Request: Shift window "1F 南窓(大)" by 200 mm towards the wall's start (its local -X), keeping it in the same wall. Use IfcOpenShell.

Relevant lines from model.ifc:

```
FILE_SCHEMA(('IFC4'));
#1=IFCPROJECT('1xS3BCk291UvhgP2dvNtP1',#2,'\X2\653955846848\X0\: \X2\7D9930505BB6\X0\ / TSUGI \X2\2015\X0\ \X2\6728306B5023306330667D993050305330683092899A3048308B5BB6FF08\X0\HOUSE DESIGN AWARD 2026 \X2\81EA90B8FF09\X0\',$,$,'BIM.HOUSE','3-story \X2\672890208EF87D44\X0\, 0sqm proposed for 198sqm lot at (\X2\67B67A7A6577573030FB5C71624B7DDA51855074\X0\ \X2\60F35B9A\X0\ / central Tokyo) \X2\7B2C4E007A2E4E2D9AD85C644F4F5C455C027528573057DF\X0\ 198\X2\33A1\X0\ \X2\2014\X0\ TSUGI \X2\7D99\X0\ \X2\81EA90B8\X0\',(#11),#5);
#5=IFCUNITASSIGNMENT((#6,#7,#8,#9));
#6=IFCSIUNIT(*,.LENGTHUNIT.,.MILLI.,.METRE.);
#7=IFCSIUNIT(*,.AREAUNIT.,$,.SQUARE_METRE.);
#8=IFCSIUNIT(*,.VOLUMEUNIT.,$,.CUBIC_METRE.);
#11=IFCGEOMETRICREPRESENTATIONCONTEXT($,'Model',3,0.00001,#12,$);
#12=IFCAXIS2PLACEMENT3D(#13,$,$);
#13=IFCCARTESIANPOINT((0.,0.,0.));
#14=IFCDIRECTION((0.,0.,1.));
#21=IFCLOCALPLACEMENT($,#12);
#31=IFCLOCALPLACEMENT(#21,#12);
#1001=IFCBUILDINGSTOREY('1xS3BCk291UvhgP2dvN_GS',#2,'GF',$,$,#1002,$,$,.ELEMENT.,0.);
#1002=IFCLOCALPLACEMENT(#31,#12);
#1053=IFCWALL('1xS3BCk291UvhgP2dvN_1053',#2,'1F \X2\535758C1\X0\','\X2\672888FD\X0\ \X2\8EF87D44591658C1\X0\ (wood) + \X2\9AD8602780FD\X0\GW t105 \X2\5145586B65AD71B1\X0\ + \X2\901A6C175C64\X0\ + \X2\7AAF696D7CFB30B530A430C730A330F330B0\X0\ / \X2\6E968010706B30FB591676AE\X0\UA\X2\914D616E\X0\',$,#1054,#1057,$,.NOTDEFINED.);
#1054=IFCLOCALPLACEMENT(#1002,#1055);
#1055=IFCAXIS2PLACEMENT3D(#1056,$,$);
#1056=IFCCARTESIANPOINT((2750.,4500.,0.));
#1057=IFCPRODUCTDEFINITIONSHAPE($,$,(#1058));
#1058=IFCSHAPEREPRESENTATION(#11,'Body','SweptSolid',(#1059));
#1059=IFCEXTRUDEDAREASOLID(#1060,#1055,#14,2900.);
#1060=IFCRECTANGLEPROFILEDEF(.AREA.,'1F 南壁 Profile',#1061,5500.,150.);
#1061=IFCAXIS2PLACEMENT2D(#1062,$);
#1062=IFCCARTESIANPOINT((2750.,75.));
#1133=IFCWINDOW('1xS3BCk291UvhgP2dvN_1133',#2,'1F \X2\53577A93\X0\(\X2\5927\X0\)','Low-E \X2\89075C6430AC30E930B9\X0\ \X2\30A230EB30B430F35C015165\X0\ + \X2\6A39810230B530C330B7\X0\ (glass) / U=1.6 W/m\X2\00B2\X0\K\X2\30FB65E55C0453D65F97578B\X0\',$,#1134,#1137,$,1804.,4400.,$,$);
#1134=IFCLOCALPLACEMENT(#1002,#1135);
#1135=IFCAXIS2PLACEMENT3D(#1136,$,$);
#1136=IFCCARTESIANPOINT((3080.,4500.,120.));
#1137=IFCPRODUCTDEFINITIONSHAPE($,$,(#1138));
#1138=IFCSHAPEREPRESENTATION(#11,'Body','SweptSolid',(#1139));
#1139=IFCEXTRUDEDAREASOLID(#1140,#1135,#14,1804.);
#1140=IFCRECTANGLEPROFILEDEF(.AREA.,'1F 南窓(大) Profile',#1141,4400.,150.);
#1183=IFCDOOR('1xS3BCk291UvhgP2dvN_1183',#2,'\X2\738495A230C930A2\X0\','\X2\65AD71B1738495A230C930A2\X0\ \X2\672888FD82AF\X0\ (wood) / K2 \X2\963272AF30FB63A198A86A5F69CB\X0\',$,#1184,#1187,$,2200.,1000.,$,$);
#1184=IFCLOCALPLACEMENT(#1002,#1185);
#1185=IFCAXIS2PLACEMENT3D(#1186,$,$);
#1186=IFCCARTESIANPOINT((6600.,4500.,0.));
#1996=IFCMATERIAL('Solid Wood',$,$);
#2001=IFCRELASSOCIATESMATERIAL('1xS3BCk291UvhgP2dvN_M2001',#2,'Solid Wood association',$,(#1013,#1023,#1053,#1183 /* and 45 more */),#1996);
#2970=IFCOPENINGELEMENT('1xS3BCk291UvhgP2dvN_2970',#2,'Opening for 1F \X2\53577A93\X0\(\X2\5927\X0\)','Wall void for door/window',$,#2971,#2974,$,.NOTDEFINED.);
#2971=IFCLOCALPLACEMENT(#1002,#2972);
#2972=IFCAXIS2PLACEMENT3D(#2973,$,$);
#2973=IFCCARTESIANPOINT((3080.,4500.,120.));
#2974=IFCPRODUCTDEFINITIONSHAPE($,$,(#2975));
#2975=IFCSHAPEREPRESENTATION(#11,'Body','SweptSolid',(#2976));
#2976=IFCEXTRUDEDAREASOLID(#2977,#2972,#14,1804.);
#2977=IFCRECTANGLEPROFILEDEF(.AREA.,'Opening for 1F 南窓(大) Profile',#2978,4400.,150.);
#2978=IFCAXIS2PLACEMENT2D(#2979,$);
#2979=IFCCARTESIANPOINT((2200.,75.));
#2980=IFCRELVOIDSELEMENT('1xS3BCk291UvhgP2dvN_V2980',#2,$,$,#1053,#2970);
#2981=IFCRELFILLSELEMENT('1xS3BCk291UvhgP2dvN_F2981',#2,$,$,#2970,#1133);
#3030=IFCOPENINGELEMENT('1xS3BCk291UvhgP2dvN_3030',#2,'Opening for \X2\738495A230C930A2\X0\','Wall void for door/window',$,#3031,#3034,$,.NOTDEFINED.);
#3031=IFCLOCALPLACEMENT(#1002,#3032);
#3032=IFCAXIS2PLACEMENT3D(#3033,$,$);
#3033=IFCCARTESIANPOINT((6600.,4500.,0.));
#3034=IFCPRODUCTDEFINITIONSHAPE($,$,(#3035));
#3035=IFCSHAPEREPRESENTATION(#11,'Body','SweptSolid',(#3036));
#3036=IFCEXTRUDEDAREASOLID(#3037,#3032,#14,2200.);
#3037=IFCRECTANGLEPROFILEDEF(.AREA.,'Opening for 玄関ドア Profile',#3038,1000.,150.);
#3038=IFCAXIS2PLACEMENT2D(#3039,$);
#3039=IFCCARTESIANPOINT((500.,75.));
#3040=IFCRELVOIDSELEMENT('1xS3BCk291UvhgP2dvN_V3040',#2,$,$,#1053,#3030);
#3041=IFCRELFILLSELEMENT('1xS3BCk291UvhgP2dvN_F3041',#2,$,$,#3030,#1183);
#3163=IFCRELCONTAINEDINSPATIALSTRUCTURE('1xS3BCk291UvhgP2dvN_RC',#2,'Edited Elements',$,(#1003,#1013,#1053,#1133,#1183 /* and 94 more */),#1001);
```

```python
import ifcopenshell
import ifcopenshell.api.geometry
import ifcopenshell.util.placement
import ifcopenshell.util.unit

model = ifcopenshell.open("model.ifc")
unit_scale = ifcopenshell.util.unit.calculate_unit_scale(model)

window = model.by_guid("1xS3BCk291UvhgP2dvN_1133")
opening = window.FillsVoids[0].RelatingOpeningElement
wall = opening.VoidsElements[0].RelatingBuildingElement

wall_matrix = ifcopenshell.util.placement.get_local_placement(wall.ObjectPlacement)
shift = wall_matrix[:3, 0] * -0.2 / unit_scale
before = ifcopenshell.util.placement.get_local_placement(window.ObjectPlacement)[:3, 3].copy()

# The window is not placed relative to its opening, so move both.
for product in (opening, window):
    matrix = ifcopenshell.util.placement.get_local_placement(product.ObjectPlacement)
    matrix[:3, 3] += shift
    ifcopenshell.api.geometry.edit_object_placement(model, product=product, matrix=matrix, is_si=False)

after = ifcopenshell.util.placement.get_local_placement(window.ObjectPlacement)[:3, 3]
print("window moved by", (after - before).round(3) + 0.0)

model.write("model_updated.ifc")
```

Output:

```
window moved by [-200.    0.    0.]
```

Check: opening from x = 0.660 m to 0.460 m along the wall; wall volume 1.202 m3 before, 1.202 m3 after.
